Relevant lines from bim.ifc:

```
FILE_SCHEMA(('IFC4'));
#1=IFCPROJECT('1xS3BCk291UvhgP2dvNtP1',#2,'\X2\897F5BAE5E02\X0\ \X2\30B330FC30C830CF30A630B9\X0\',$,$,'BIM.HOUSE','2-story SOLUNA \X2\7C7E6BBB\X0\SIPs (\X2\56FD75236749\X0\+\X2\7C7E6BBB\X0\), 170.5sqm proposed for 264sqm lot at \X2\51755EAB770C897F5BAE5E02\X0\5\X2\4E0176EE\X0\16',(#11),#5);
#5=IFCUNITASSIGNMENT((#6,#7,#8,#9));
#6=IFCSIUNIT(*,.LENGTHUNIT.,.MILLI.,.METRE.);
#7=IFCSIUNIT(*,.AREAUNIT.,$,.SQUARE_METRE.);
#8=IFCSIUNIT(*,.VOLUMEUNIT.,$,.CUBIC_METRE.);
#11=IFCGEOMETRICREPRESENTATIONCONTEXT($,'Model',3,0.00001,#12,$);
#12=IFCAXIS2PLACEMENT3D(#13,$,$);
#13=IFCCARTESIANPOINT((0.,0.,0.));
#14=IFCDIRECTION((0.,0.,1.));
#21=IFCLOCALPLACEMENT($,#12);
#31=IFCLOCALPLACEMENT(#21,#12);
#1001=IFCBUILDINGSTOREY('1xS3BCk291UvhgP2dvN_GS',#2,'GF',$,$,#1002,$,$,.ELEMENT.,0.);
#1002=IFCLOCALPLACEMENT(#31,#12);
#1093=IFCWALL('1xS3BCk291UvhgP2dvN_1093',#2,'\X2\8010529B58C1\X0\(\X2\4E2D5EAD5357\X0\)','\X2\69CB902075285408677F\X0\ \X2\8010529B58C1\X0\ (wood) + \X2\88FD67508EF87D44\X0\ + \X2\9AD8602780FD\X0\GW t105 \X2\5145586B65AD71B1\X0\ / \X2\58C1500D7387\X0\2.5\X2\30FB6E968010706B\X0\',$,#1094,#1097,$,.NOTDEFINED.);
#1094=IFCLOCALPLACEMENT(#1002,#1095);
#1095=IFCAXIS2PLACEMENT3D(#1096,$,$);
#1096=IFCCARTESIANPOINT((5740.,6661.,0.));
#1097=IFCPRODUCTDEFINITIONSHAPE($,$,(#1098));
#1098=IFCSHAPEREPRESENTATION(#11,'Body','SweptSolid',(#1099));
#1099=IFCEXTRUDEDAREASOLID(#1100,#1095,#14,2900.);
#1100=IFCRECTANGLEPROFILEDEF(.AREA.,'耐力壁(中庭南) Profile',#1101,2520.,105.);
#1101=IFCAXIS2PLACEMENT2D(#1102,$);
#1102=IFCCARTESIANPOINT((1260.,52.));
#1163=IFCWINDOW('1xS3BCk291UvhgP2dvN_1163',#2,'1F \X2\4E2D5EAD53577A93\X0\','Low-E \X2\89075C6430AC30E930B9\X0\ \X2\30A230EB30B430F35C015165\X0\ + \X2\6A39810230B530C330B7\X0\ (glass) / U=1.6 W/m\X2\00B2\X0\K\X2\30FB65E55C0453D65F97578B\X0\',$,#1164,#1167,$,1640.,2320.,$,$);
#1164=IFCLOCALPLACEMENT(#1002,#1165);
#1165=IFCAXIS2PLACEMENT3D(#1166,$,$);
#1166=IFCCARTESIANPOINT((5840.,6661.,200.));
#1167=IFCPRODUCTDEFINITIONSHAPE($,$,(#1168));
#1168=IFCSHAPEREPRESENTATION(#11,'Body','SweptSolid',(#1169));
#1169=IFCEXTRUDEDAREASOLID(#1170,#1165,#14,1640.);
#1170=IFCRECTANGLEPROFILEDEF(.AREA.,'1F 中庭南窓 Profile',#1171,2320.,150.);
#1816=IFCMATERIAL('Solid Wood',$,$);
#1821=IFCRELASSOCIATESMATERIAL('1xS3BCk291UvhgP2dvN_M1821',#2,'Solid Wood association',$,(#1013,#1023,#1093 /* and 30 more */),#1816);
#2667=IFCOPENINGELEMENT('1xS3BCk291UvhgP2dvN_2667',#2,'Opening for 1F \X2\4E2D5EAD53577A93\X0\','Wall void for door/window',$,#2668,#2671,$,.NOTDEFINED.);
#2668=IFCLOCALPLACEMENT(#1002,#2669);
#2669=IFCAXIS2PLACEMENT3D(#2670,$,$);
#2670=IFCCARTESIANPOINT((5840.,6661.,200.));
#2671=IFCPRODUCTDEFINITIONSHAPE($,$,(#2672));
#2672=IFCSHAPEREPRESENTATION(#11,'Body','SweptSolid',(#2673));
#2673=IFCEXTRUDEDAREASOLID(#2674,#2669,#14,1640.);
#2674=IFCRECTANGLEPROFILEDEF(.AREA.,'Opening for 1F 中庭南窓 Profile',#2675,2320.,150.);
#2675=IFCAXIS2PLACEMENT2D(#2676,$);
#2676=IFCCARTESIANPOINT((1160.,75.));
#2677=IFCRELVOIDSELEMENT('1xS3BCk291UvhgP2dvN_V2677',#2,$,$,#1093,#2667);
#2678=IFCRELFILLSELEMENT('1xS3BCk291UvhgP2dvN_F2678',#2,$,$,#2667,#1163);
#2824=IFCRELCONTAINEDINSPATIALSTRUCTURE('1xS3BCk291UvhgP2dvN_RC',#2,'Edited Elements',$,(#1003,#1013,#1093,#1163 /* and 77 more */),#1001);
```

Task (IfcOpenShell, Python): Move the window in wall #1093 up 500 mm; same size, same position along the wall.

```python
import numpy as np
import ifcopenshell
import ifcopenshell.api.geometry
import ifcopenshell.util.placement
import ifcopenshell.util.unit

model = ifcopenshell.open("bim.ifc")
unit_scale = ifcopenshell.util.unit.calculate_unit_scale(model)

window = model.by_id(1163)
opening = window.FillsVoids[0].RelatingOpeningElement
dz = 0.5 / unit_scale

shift = np.array([0.0, 0.0, dz])
# The window is not placed relative to its opening, so move both.
for product in (opening, window):
    matrix = ifcopenshell.util.placement.get_local_placement(product.ObjectPlacement)
    matrix[:3, 3] += shift
    ifcopenshell.api.geometry.edit_object_placement(model, product=product, matrix=matrix, is_si=False)

print(f"moved by {dz * unit_scale:+.3f} m")

model.write("bim-out.ifc")
```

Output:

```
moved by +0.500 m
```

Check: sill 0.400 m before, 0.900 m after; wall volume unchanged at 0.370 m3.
